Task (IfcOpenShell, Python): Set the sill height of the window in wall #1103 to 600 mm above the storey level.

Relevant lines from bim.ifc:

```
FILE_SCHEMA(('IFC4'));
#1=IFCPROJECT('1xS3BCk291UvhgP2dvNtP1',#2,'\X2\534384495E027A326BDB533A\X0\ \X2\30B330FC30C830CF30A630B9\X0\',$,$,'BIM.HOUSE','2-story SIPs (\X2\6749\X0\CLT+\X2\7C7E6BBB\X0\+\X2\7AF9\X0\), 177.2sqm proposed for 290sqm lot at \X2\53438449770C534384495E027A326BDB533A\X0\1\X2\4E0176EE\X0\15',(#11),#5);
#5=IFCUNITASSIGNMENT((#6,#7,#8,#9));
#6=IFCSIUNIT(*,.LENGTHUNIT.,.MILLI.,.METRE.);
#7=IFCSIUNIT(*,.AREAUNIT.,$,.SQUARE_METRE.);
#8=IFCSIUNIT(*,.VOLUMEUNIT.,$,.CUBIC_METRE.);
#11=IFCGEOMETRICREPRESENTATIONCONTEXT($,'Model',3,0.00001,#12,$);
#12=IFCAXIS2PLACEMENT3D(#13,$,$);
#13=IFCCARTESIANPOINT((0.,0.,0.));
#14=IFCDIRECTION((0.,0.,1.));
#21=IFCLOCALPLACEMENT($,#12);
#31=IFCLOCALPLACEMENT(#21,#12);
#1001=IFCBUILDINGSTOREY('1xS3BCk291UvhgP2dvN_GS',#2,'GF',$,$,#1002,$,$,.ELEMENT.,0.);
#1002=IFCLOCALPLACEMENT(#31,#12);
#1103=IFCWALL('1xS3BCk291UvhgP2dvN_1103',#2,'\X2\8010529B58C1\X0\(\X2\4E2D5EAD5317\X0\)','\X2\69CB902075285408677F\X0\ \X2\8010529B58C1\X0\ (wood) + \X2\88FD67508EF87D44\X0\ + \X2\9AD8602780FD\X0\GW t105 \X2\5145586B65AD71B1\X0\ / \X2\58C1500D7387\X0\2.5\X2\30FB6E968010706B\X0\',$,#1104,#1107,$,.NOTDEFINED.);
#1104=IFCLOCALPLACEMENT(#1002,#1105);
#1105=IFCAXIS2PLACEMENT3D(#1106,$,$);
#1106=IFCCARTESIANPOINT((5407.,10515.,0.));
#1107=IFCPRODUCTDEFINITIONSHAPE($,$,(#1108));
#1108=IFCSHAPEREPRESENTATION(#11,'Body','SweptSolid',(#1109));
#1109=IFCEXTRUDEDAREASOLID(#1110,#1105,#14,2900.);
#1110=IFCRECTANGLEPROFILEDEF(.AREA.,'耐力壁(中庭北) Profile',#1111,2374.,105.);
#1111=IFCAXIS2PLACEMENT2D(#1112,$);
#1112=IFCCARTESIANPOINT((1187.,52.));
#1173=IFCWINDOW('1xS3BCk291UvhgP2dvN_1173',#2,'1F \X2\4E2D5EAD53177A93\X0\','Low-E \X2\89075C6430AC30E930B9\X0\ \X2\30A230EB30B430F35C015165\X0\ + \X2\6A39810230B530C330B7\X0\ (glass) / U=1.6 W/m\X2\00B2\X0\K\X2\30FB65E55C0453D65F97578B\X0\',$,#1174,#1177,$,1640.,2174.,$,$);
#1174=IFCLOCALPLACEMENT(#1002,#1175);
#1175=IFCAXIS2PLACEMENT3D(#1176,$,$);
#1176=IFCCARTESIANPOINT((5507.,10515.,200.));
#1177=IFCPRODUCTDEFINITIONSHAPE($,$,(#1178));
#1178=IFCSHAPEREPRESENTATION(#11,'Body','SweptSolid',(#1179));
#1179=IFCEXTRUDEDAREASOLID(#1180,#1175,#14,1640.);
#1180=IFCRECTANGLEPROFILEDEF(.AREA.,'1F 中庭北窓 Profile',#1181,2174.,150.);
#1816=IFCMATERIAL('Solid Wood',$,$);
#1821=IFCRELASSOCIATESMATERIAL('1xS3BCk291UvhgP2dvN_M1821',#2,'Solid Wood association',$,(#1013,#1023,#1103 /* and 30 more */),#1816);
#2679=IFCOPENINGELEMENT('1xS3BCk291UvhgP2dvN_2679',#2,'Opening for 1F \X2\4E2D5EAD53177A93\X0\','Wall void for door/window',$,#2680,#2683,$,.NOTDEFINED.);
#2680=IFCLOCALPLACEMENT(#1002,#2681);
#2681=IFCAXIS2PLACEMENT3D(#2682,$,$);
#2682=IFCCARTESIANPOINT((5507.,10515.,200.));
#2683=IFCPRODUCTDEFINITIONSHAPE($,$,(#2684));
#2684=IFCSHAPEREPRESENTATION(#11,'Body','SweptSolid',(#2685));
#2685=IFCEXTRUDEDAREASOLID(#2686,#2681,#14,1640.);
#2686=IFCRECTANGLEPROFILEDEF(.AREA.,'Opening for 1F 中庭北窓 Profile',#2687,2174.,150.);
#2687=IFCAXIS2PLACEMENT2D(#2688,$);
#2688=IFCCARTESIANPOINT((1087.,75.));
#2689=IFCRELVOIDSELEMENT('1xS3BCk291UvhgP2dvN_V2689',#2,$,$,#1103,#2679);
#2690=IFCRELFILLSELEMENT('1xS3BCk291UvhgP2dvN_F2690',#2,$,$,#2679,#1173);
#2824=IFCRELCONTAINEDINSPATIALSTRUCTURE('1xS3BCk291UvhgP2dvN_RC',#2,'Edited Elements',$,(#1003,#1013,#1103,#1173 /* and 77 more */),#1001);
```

```python
import numpy as np
import ifcopenshell
import ifcopenshell.api.geometry
import ifcopenshell.geom
import ifcopenshell.util.element
import ifcopenshell.util.placement
import ifcopenshell.util.shape
import ifcopenshell.util.unit

model = ifcopenshell.open("bim.ifc")
unit_scale = ifcopenshell.util.unit.calculate_unit_scale(model)

window = model.by_guid("1xS3BCk291UvhgP2dvN_1173")
opening = window.FillsVoids[0].RelatingOpeningElement
storey = ifcopenshell.util.element.get_container(window, ifc_class="IfcBuildingStorey")
level = ifcopenshell.util.placement.get_local_placement(storey.ObjectPlacement)[2, 3]

# The opening's origin need not be at the sill, so measure its lowest point.
shape = ifcopenshell.geom.create_shape(ifcopenshell.geom.settings(), opening)
bottom = ifcopenshell.util.shape.get_shape_bottom_elevation(shape, shape.geometry) / unit_scale
dz = level + 0.6 / unit_scale - bottom

shift = np.array([0.0, 0.0, dz])
# The window is not placed relative to its opening, so move both.
for product in (opening, window):
    matrix = ifcopenshell.util.placement.get_local_placement(product.ObjectPlacement)
    matrix[:3, 3] += shift
    ifcopenshell.api.geometry.edit_object_placement(model, product=product, matrix=matrix, is_si=False)

print(f"moved by {dz * unit_scale:+.3f} m")

model.write("bim_rev.ifc")
```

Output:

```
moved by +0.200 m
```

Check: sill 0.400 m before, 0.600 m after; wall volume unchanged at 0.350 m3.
